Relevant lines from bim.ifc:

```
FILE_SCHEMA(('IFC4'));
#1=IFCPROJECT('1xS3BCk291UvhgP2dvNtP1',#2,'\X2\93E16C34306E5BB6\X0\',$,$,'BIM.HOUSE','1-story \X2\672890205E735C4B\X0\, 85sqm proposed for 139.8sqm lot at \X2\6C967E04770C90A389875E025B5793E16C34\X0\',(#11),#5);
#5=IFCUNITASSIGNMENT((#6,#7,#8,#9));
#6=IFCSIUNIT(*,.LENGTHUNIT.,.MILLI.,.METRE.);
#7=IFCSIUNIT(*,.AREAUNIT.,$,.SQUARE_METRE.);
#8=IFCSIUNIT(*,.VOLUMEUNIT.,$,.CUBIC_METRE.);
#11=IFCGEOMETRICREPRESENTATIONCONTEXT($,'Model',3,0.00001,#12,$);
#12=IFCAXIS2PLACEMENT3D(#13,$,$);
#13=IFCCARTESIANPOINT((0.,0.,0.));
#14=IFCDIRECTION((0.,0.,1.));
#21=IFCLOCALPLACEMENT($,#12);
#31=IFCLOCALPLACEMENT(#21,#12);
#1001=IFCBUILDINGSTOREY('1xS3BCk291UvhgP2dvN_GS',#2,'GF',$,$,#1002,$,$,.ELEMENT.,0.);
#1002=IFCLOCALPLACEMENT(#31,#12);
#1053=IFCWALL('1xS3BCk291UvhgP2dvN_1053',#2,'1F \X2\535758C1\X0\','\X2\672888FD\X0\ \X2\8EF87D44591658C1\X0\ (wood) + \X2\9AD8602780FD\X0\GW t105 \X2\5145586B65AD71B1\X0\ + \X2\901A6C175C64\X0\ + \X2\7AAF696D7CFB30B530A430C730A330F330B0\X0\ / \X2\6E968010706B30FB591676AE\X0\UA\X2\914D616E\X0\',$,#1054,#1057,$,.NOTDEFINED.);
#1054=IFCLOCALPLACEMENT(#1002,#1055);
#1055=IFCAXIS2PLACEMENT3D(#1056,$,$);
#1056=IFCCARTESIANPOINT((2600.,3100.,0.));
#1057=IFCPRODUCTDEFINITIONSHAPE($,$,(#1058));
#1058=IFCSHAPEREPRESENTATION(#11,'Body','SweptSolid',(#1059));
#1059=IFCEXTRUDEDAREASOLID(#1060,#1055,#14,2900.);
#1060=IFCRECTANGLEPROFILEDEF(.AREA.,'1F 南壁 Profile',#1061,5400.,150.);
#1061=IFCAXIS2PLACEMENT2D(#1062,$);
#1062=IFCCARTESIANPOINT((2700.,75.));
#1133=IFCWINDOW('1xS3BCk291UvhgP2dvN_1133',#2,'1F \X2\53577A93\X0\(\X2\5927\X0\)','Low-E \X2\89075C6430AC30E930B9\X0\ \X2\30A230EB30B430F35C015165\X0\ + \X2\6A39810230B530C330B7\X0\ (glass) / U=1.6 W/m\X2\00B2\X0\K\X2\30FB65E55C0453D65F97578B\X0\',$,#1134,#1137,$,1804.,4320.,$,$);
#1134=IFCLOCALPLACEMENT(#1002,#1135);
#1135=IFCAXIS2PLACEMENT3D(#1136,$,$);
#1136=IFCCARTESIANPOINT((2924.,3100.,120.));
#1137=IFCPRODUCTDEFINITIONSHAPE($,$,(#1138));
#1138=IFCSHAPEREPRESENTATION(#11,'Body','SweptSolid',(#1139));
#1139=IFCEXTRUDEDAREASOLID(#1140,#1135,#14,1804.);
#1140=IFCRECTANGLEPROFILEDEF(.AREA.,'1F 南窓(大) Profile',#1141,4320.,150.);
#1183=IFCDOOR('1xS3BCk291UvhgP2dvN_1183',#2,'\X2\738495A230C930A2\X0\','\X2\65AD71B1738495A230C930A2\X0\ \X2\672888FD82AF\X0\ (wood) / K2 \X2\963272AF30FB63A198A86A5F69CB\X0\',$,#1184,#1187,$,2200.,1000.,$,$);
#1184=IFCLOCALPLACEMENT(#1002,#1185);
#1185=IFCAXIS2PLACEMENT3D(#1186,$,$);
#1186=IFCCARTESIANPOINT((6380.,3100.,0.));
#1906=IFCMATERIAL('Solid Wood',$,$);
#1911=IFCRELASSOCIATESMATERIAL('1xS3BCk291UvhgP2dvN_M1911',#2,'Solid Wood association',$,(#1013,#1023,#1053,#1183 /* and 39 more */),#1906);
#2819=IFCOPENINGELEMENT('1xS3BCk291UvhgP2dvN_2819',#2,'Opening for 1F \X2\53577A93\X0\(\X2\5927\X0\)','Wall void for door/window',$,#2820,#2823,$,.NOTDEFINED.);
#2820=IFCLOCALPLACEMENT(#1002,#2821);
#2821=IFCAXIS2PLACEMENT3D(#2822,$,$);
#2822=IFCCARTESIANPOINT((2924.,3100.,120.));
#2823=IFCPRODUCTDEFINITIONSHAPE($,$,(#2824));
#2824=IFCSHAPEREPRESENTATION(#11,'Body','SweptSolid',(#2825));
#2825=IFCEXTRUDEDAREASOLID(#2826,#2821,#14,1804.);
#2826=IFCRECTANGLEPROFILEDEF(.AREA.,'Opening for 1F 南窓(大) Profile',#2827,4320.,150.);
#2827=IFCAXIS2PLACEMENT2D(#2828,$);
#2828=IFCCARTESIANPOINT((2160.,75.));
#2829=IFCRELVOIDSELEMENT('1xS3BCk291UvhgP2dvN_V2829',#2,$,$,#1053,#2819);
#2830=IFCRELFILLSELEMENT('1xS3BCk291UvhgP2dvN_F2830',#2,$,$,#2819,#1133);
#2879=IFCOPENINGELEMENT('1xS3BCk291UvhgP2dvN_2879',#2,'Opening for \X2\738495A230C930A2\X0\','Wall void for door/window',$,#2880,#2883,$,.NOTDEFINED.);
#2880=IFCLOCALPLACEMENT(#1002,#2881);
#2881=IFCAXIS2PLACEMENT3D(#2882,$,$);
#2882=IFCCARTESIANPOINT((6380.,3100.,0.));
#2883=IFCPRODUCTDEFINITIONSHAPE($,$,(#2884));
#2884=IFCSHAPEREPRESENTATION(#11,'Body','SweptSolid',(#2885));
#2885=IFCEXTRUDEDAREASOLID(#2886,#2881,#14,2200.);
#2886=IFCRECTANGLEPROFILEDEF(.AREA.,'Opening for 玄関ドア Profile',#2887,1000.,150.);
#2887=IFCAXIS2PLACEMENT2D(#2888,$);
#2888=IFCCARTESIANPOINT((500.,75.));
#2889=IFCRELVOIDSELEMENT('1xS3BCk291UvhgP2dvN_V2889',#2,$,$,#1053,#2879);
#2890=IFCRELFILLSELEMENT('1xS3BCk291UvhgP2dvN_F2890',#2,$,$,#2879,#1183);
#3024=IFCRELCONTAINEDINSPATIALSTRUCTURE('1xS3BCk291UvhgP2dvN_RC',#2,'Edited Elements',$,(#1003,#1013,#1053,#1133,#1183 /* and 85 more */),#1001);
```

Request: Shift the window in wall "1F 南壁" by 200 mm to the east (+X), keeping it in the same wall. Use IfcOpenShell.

```python
import ifcopenshell
import ifcopenshell.api.geometry
import ifcopenshell.util.placement
import ifcopenshell.util.unit

model = ifcopenshell.open("bim.ifc")
unit_scale = ifcopenshell.util.unit.calculate_unit_scale(model)

window = model.by_guid("1xS3BCk291UvhgP2dvN_1133")
opening = window.FillsVoids[0].RelatingOpeningElement
wall = opening.VoidsElements[0].RelatingBuildingElement

wall_matrix = ifcopenshell.util.placement.get_local_placement(wall.ObjectPlacement)
shift = wall_matrix[:3, 0] * 0.2 / unit_scale
before = ifcopenshell.util.placement.get_local_placement(window.ObjectPlacement)[:3, 3].copy()

# The window is not placed relative to its opening, so move both.
for product in (opening, window):
    matrix = ifcopenshell.util.placement.get_local_placement(product.ObjectPlacement)
    matrix[:3, 3] += shift
    ifcopenshell.api.geometry.edit_object_placement(model, product=product, matrix=matrix, is_si=False)

after = ifcopenshell.util.placement.get_local_placement(window.ObjectPlacement)[:3, 3]
print("window moved by", (after - before).round(3) + 0.0)

model.write("bim-out.ifc")
```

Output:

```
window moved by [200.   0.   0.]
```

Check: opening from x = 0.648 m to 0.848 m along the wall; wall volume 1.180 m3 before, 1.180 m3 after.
